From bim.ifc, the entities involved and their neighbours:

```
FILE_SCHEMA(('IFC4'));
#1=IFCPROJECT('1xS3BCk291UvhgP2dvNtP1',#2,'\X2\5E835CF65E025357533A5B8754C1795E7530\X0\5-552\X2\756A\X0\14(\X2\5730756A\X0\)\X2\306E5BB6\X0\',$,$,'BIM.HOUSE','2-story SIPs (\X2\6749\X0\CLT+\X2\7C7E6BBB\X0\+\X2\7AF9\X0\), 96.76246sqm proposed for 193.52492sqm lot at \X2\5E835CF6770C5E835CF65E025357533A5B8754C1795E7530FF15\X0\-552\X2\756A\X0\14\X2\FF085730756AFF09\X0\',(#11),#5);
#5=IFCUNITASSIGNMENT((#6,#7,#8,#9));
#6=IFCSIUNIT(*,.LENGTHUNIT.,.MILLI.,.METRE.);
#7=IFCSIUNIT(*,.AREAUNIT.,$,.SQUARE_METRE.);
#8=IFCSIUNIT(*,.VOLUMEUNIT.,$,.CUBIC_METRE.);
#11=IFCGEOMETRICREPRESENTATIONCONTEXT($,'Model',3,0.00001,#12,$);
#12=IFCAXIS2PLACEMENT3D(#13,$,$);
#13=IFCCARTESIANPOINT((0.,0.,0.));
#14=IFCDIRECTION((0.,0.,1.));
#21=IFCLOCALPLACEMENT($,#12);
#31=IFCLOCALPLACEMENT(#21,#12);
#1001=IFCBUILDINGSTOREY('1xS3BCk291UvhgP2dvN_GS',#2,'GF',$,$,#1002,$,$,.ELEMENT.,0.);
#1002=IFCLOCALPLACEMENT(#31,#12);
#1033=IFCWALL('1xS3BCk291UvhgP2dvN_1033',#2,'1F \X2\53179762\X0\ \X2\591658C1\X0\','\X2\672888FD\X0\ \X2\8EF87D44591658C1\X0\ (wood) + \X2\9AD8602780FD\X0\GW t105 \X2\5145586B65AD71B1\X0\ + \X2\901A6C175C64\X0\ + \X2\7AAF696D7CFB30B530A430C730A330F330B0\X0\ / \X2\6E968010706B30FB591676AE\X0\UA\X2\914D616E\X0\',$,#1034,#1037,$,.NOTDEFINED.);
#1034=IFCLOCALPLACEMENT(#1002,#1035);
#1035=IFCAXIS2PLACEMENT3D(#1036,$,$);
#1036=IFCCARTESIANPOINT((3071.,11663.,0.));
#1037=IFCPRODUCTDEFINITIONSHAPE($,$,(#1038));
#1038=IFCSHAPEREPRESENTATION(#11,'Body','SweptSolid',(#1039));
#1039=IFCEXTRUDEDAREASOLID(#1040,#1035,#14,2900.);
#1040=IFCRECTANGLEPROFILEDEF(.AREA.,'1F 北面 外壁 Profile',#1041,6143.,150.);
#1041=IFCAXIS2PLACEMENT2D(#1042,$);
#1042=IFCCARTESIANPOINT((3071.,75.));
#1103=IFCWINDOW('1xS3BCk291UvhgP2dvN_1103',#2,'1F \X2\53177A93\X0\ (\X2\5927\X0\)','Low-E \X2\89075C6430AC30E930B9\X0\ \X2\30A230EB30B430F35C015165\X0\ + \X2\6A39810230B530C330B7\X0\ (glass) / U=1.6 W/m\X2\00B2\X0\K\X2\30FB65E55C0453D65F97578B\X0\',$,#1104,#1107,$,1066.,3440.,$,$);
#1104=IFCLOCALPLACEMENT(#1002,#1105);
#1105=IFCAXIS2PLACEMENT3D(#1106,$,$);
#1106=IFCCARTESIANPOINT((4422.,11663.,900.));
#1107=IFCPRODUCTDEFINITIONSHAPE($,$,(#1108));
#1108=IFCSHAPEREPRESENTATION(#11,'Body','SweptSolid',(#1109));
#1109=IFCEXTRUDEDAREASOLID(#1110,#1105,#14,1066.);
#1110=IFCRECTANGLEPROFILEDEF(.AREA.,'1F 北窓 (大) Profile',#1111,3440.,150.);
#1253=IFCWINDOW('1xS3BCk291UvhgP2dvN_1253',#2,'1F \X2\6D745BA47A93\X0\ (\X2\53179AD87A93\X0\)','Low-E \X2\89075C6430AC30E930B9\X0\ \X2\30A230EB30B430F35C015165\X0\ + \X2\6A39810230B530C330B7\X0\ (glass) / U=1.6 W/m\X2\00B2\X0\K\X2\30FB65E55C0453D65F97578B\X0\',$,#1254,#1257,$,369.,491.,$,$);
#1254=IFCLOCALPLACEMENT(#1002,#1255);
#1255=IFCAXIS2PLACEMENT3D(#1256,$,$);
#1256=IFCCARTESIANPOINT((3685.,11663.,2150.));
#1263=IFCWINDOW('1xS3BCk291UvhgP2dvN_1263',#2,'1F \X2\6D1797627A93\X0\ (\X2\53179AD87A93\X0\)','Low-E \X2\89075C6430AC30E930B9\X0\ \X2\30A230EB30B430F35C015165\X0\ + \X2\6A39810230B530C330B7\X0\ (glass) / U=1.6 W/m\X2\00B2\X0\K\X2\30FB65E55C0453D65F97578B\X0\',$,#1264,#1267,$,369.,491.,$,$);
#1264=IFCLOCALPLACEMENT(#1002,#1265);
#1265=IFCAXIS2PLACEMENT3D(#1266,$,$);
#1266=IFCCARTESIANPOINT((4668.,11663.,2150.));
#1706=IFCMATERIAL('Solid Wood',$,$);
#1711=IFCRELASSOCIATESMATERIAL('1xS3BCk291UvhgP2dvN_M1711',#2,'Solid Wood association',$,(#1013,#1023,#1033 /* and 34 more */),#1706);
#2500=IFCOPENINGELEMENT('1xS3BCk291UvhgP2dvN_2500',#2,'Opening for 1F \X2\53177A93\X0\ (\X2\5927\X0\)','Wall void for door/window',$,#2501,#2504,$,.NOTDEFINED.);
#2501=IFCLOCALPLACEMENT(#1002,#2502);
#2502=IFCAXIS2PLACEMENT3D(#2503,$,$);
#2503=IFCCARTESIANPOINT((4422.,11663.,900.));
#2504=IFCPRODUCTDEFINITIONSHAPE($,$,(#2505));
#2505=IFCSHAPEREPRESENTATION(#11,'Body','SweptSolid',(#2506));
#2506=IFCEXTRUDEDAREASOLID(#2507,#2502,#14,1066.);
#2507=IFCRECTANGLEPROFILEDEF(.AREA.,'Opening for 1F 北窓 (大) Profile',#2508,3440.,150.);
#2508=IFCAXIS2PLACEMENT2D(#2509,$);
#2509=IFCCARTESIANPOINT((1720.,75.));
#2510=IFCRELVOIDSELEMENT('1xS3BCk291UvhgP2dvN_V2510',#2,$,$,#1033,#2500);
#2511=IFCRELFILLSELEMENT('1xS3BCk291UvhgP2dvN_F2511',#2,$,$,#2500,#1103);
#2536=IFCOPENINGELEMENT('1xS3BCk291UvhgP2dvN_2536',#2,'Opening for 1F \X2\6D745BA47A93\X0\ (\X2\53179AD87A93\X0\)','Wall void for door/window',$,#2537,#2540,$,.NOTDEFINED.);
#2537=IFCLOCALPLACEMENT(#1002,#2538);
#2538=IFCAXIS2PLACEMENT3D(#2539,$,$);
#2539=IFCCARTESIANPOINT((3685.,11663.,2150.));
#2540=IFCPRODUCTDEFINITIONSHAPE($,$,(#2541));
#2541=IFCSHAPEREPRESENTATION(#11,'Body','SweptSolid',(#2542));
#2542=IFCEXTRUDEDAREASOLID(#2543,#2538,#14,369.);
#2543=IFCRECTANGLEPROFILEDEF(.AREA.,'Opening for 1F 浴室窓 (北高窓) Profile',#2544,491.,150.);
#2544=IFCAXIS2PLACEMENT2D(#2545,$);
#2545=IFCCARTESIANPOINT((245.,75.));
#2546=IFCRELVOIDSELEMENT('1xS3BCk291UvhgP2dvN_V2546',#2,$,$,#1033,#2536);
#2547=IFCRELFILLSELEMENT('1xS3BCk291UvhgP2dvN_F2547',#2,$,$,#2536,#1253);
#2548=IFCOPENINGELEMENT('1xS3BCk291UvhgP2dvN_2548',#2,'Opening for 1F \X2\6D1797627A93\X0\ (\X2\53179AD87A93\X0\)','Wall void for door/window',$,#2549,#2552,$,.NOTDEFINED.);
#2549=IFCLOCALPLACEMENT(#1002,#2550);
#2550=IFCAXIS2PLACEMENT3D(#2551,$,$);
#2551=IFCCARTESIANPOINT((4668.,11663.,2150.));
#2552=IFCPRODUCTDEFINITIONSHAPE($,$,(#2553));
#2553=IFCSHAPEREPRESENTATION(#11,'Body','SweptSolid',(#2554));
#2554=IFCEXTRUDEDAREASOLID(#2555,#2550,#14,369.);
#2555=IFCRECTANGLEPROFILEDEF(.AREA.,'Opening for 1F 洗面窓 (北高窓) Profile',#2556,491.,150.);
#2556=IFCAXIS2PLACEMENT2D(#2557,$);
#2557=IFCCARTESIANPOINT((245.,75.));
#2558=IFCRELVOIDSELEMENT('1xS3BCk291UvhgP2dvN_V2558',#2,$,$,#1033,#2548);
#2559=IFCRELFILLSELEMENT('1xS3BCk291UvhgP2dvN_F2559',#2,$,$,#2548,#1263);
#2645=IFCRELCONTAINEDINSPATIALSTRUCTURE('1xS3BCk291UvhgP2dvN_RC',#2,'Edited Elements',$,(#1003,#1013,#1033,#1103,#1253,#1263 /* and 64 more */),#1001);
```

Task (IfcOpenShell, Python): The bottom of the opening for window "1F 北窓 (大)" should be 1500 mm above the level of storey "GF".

```python
import numpy as np
import ifcopenshell
import ifcopenshell.api.geometry
import ifcopenshell.geom
import ifcopenshell.util.element
import ifcopenshell.util.placement
import ifcopenshell.util.shape
import ifcopenshell.util.unit

model = ifcopenshell.open("bim.ifc")
unit_scale = ifcopenshell.util.unit.calculate_unit_scale(model)

window = model.by_guid("1xS3BCk291UvhgP2dvN_1103")
opening = window.FillsVoids[0].RelatingOpeningElement
storey = ifcopenshell.util.element.get_container(window, ifc_class="IfcBuildingStorey")
level = ifcopenshell.util.placement.get_local_placement(storey.ObjectPlacement)[2, 3]

# The opening's origin need not be at the sill, so measure its lowest point.
shape = ifcopenshell.geom.create_shape(ifcopenshell.geom.settings(), opening)
bottom = ifcopenshell.util.shape.get_shape_bottom_elevation(shape, shape.geometry) / unit_scale
dz = level + 1.5 / unit_scale - bottom

shift = np.array([0.0, 0.0, dz])
# The window is not placed relative to its opening, so move both.
for product in (opening, window):
    matrix = ifcopenshell.util.placement.get_local_placement(product.ObjectPlacement)
    matrix[:3, 3] += shift
    ifcopenshell.api.geometry.edit_object_placement(model, product=product, matrix=matrix, is_si=False)

print(f"moved by {dz * unit_scale:+.3f} m")

model.write("bim-out.ifc")
```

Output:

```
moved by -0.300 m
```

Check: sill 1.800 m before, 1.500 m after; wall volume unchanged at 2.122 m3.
